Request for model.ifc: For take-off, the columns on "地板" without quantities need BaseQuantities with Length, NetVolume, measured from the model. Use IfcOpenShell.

First a look at what the model holds.

```python
import ifcopenshell
import ifcopenshell.util.element
import ifcopenshell.util.unit

model = ifcopenshell.open("model.ifc")
print(model.schema)
for unit_type in ("LENGTHUNIT", "AREAUNIT", "VOLUMEUNIT"):
    print(unit_type, ifcopenshell.util.unit.calculate_unit_scale(model, unit_type))
storey = next(s for s in model.by_type("IfcBuildingStorey") if s.Name == "地板")
columns = [e for e in ifcopenshell.util.element.get_decomposition(storey) if e.is_a("IfcColumn")]
for e in sorted(columns, key=lambda e: e.id()):
    print(e.id(), e.is_a(), e.Name, list(ifcopenshell.util.element.get_psets(e, qtos_only=True)), sep=" | ")
```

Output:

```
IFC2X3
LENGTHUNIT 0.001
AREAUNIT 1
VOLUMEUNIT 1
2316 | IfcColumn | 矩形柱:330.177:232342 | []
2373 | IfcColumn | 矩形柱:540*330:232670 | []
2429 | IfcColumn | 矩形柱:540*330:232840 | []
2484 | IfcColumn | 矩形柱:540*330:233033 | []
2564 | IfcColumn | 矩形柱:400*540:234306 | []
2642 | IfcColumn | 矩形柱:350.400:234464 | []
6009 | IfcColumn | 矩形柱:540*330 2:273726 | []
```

```python
import ifcopenshell
import ifcopenshell.api.pset
import ifcopenshell.geom
import ifcopenshell.util.element
import ifcopenshell.util.shape
import ifcopenshell.util.unit

model = ifcopenshell.open("model.ifc")
unit_scale = ifcopenshell.util.unit.calculate_unit_scale(model)
volume_scale = ifcopenshell.util.unit.calculate_unit_scale(model, "VOLUMEUNIT")
settings = ifcopenshell.geom.settings()

storey = next(s for s in model.by_type("IfcBuildingStorey") if s.Name == "地板")
columns = [e for e in ifcopenshell.util.element.get_decomposition(storey) if e.is_a("IfcColumn")]

for e in sorted(columns, key=lambda e: e.id()):
    if ifcopenshell.util.element.get_psets(e, qtos_only=True, should_inherit=False):
        continue
    # Geometry comes back in metres, in the element's own axes.
    shape = ifcopenshell.geom.create_shape(settings, e)
    values = {
        "Length": ifcopenshell.util.shape.get_z(shape.geometry) / unit_scale,
        "NetVolume": ifcopenshell.util.shape.get_volume(shape.geometry) / volume_scale,
    }
    qto = ifcopenshell.api.pset.add_qto(model, product=e, name="BaseQuantities")
    ifcopenshell.api.pset.edit_qto(model, qto=qto, properties=values)
    print(e.id(), {k: round(v, 3) for k, v in values.items()})

model.write("model_edited.ifc")
```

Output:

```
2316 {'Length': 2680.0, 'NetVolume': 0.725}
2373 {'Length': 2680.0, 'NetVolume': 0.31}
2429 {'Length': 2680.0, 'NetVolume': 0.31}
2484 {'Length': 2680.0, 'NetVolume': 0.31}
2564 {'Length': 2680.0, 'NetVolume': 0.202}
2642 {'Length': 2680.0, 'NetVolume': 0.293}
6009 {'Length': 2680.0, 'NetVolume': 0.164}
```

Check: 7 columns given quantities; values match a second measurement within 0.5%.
